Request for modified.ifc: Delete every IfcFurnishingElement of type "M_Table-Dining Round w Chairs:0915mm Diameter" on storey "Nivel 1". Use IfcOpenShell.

First a look at what the model holds.

```python
import ifcopenshell
import ifcopenshell.util.element

model = ifcopenshell.open("modified.ifc")
print(model.schema)
storey = next(s for s in model.by_type("IfcBuildingStorey") if s.Name == "Nivel 1")
furniture = [e for e in ifcopenshell.util.element.get_decomposition(storey) if e.is_a("IfcFurnishingElement")]
seen = {}
for e in furniture:
    element_type = ifcopenshell.util.element.get_type(e)
    name = element_type.Name if element_type not in (None, e) else None
    seen[name] = seen.get(name, 0) + 1
for name, count in sorted(seen.items(), key=str):
    print(count, "x", name)
```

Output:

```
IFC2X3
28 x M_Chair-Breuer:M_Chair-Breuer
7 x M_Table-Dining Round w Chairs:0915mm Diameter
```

```python
import ifcopenshell
import ifcopenshell.api.root
import ifcopenshell.util.element

model = ifcopenshell.open("modified.ifc")

storey = next(s for s in model.by_type("IfcBuildingStorey") if s.Name == "Nivel 1")
furniture = [e for e in ifcopenshell.util.element.get_decomposition(storey) if e.is_a("IfcFurnishingElement")]
targets = [e for e in furniture if (t := ifcopenshell.util.element.get_type(e)) not in (None, e) and t.Name == "M_Table-Dining Round w Chairs:0915mm Diameter"]

for e in targets:
    ifcopenshell.api.root.remove_product(model, product=e)
print(len(targets), "removed")

model.write("modified_v2.ifc")
```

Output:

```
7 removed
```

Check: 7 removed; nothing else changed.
